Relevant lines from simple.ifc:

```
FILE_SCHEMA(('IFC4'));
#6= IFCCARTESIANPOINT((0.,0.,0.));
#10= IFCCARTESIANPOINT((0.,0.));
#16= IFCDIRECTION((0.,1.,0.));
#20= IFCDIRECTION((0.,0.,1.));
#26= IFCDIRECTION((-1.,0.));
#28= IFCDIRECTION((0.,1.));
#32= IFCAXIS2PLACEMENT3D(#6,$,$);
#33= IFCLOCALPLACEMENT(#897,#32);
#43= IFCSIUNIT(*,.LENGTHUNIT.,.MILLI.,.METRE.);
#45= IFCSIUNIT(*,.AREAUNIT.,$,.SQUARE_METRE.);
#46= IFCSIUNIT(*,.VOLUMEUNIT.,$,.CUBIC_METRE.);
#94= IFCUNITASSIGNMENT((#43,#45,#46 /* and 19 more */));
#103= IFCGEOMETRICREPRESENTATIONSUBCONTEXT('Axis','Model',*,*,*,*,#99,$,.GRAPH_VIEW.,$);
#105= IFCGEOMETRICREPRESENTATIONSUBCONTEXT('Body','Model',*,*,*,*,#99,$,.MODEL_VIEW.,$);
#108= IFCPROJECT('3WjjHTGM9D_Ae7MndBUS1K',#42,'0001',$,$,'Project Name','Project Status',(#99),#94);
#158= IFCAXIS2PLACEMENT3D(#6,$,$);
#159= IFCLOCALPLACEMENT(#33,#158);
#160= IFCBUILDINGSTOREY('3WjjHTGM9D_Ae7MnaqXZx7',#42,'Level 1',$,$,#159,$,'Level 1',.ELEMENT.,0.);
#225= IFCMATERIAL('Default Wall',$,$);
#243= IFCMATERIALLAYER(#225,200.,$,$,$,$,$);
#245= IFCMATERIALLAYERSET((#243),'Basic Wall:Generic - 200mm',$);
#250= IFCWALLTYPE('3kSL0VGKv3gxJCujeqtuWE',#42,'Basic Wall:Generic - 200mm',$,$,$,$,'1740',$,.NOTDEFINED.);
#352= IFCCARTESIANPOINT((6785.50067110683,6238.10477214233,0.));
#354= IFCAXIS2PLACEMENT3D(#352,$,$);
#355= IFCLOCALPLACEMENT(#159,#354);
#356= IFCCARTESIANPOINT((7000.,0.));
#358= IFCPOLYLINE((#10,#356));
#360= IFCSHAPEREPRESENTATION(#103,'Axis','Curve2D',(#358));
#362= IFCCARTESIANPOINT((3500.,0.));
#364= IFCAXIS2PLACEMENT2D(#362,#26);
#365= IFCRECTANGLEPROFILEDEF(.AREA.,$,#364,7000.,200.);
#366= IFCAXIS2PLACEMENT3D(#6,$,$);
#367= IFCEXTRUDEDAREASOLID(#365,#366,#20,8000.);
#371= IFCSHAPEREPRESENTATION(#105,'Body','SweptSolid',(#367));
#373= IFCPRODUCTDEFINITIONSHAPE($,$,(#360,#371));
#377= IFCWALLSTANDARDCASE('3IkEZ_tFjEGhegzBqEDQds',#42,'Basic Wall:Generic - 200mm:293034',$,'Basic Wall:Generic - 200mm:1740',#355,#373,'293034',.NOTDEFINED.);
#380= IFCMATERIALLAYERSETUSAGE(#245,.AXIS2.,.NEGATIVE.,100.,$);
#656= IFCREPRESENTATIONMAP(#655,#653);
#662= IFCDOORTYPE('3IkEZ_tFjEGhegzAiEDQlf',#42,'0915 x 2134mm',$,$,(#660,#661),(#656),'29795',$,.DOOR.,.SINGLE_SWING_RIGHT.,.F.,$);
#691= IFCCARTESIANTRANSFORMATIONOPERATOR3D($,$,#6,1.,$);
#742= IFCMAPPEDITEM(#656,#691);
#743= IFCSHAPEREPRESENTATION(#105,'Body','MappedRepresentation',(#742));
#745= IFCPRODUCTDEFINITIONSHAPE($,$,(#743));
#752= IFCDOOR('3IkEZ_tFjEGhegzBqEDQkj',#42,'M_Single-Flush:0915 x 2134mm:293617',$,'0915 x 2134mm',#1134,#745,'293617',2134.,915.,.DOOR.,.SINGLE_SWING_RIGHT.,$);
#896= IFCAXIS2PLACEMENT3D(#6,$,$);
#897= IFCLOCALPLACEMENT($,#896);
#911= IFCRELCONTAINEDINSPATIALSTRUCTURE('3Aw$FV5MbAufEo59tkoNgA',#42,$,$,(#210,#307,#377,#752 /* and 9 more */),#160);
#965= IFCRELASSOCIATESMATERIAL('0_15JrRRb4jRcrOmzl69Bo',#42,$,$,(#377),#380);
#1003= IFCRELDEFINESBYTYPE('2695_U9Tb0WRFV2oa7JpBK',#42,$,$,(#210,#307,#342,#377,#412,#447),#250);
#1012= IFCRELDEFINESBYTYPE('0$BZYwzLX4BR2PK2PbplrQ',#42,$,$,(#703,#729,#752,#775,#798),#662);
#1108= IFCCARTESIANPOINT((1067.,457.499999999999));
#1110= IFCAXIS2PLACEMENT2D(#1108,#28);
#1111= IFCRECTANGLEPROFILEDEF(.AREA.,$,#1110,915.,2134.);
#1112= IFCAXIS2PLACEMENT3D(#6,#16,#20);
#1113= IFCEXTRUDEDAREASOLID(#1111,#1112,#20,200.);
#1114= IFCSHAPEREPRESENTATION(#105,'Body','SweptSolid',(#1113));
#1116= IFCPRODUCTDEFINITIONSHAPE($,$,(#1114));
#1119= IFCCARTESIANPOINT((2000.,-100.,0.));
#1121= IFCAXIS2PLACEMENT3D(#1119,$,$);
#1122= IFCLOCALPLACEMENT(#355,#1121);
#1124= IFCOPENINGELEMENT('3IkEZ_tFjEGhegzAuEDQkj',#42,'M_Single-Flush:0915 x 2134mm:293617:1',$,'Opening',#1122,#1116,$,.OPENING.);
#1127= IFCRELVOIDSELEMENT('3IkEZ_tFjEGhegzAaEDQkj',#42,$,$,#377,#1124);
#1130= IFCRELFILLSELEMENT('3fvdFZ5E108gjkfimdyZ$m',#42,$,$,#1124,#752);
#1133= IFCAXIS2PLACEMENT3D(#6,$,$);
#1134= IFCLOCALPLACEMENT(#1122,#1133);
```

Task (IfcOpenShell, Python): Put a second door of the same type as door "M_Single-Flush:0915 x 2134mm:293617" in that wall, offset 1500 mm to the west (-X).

```python
import ifcopenshell
import ifcopenshell.api.feature
import ifcopenshell.api.geometry
import ifcopenshell.api.root
import ifcopenshell.geom
import ifcopenshell.util.element
import ifcopenshell.util.placement
import ifcopenshell.util.shape
import ifcopenshell.util.unit

model = ifcopenshell.open("simple.ifc")
unit_scale = ifcopenshell.util.unit.calculate_unit_scale(model)
settings = ifcopenshell.geom.settings()


def volume(element):
    """Net volume in cubic metres, openings subtracted."""
    shape = ifcopenshell.geom.create_shape(settings, element)
    return ifcopenshell.util.shape.get_volume(shape.geometry)


def reuse_history(source, copy):
    """copy_class also copies each property set's owner history, people and application; keep the originals."""
    for rel in copy.IsDefinedBy:
        if rel.is_a("IfcRelDefinesByProperties") and (history := rel.RelatingPropertyDefinition.OwnerHistory):
            rel.RelatingPropertyDefinition.OwnerHistory = source.OwnerHistory
            ifcopenshell.util.element.remove_deep2(model, history)


door = model.by_guid("3IkEZ_tFjEGhegzBqEDQkj")
opening = door.FillsVoids[0].RelatingOpeningElement
wall = opening.VoidsElements[0].RelatingBuildingElement
before = volume(wall)
shift = ifcopenshell.util.placement.get_local_placement(wall.ObjectPlacement)[:3, 0] * -1.5 / unit_scale

# copy_class copies the void relationship, type, container and properties, but no geometry.
new_opening = ifcopenshell.api.root.copy_class(model, product=opening)
new_opening.Representation = ifcopenshell.util.element.copy_deep(
    model, opening.Representation, exclude=["IfcGeometricRepresentationContext", "IfcRepresentationMap"]
)
new_opening.Name = "M_Single-Flush:0915 x 2134mm"
new_door = ifcopenshell.api.root.copy_class(model, product=door)
new_door.Representation = ifcopenshell.util.element.copy_deep(
    model, door.Representation, exclude=["IfcGeometricRepresentationContext", "IfcRepresentationMap"]
)
new_door.Name = "M_Single-Flush:0915 x 2134mm"
new_door.Tag = None
reuse_history(door, new_door)
ifcopenshell.api.feature.add_filling(model, opening=new_opening, element=new_door)

for old, new in ((opening, new_opening), (door, new_door)):
    matrix = ifcopenshell.util.placement.get_local_placement(old.ObjectPlacement)
    matrix[:3, 3] += shift
    ifcopenshell.api.geometry.edit_object_placement(model, product=new, matrix=matrix, is_si=False)

after = volume(wall)

print(f"wall volume {before:.3f} -> {after:.3f} m3")

model.write("simple_rev.ifc")
```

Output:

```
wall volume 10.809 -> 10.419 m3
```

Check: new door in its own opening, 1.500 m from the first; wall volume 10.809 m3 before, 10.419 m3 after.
